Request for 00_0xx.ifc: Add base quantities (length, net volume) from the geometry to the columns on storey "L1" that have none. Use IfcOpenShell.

First a look at what the model holds.

```python
import ifcopenshell
import ifcopenshell.util.element
import ifcopenshell.util.unit

model = ifcopenshell.open("00_0xx.ifc")
print(model.schema)
for unit_type in ("LENGTHUNIT", "AREAUNIT", "VOLUMEUNIT"):
    print(unit_type, ifcopenshell.util.unit.calculate_unit_scale(model, unit_type))
storey = next(s for s in model.by_type("IfcBuildingStorey") if s.Name == "L1")
columns = [e for e in ifcopenshell.util.element.get_decomposition(storey) if e.is_a("IfcColumn")]
for e in sorted(columns, key=lambda e: e.id()):
    print(e.id(), e.is_a(), e.Name, list(ifcopenshell.util.element.get_psets(e, qtos_only=True)), sep=" | ")
```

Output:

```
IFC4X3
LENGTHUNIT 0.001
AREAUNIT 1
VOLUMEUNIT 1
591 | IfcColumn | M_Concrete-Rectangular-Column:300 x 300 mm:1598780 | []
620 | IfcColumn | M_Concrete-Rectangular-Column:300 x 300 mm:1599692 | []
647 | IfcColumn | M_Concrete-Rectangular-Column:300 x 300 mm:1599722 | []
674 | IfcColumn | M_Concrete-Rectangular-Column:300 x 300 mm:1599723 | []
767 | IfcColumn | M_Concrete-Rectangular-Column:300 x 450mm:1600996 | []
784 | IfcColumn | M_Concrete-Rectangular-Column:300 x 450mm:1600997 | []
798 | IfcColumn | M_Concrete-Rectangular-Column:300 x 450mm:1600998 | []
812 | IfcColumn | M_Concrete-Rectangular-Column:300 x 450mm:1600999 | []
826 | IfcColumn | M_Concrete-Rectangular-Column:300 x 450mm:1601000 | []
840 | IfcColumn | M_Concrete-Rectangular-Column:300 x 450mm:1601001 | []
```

```python
import ifcopenshell
import ifcopenshell.api.pset
import ifcopenshell.geom
import ifcopenshell.util.element
import ifcopenshell.util.shape
import ifcopenshell.util.unit

model = ifcopenshell.open("00_0xx.ifc")
unit_scale = ifcopenshell.util.unit.calculate_unit_scale(model)
volume_scale = ifcopenshell.util.unit.calculate_unit_scale(model, "VOLUMEUNIT")
settings = ifcopenshell.geom.settings()

storey = next(s for s in model.by_type("IfcBuildingStorey") if s.Name == "L1")
columns = [e for e in ifcopenshell.util.element.get_decomposition(storey) if e.is_a("IfcColumn")]

for e in sorted(columns, key=lambda e: e.id()):
    if ifcopenshell.util.element.get_psets(e, qtos_only=True, should_inherit=False):
        continue
    # Geometry comes back in metres, in the element's own axes.
    shape = ifcopenshell.geom.create_shape(settings, e)
    values = {
        "Length": ifcopenshell.util.shape.get_z(shape.geometry) / unit_scale,
        "NetVolume": ifcopenshell.util.shape.get_volume(shape.geometry) / volume_scale,
    }
    qto = ifcopenshell.api.pset.add_qto(model, product=e, name="Qto_ColumnBaseQuantities")
    ifcopenshell.api.pset.edit_qto(model, qto=qto, properties=values)
    print(e.id(), {k: round(v, 3) for k, v in values.items()})

model.write("00_0xx_updated.ifc")
```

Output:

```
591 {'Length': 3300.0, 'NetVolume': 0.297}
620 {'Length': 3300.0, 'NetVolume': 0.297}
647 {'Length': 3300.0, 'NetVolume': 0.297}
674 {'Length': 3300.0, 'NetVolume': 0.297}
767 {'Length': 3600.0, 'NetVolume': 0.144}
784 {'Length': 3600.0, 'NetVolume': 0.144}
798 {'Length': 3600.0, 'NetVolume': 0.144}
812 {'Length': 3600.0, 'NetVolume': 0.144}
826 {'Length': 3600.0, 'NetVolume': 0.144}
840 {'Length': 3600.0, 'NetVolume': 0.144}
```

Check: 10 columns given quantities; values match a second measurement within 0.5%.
